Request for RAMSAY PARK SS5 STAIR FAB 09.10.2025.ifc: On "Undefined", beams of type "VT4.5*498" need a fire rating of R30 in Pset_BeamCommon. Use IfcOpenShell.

First a look at what the model holds.

```python
import ifcopenshell
import ifcopenshell.util.element

model = ifcopenshell.open("RAMSAY PARK SS5 STAIR FAB 09.10.2025.ifc")
print(model.schema)
storey = next(s for s in model.by_type("IfcBuildingStorey") if s.Name == "Undefined")
beams = [e for e in ifcopenshell.util.element.get_decomposition(storey) if e.is_a("IfcBeam")]
seen = {}
for e in beams:
    element_type = ifcopenshell.util.element.get_type(e)
    key = (element_type.Name if element_type != e and element_type else None, ifcopenshell.util.element.get_pset(e, "Pset_BeamCommon", "FireRating"))
    seen[key] = seen.get(key, 0) + 1
for (name, value), count in sorted(seen.items(), key=str):
    print(count, "x", name, "|", value)
```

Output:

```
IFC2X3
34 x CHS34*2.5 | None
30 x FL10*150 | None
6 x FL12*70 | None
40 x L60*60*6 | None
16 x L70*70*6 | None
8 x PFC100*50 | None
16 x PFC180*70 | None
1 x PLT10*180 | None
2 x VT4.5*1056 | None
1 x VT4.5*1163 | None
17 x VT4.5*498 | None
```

```python
import ifcopenshell
import ifcopenshell.api.pset
import ifcopenshell.util.element

model = ifcopenshell.open("RAMSAY PARK SS5 STAIR FAB 09.10.2025.ifc")

storey = next(s for s in model.by_type("IfcBuildingStorey") if s.Name == "Undefined")
beams = [e for e in ifcopenshell.util.element.get_decomposition(storey) if e.is_a("IfcBeam")]

count = 0
for e in beams:
    element_type = ifcopenshell.util.element.get_type(e)
    if element_type in (None, e) or element_type.Name != "VT4.5*498":
        continue
    found = ifcopenshell.util.element.get_pset(e, "Pset_BeamCommon", should_inherit=False)
    if found:
        pset = model.by_id(found["id"])
        if len(ifcopenshell.util.element.get_elements_by_pset(pset)) > 1:
            pset = ifcopenshell.api.pset.unshare_pset(model, products=[e], pset=pset)[0]
    else:
        pset = ifcopenshell.api.pset.add_pset(model, product=e, name="Pset_BeamCommon")
    ifcopenshell.api.pset.edit_pset(model, pset=pset, properties={"FireRating": "R30"})
    count += 1

print(count, "beams updated")

model.write("RAMSAY PARK SS5 STAIR FAB 09.10.2025_updated.ifc")
```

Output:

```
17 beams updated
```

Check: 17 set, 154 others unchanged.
